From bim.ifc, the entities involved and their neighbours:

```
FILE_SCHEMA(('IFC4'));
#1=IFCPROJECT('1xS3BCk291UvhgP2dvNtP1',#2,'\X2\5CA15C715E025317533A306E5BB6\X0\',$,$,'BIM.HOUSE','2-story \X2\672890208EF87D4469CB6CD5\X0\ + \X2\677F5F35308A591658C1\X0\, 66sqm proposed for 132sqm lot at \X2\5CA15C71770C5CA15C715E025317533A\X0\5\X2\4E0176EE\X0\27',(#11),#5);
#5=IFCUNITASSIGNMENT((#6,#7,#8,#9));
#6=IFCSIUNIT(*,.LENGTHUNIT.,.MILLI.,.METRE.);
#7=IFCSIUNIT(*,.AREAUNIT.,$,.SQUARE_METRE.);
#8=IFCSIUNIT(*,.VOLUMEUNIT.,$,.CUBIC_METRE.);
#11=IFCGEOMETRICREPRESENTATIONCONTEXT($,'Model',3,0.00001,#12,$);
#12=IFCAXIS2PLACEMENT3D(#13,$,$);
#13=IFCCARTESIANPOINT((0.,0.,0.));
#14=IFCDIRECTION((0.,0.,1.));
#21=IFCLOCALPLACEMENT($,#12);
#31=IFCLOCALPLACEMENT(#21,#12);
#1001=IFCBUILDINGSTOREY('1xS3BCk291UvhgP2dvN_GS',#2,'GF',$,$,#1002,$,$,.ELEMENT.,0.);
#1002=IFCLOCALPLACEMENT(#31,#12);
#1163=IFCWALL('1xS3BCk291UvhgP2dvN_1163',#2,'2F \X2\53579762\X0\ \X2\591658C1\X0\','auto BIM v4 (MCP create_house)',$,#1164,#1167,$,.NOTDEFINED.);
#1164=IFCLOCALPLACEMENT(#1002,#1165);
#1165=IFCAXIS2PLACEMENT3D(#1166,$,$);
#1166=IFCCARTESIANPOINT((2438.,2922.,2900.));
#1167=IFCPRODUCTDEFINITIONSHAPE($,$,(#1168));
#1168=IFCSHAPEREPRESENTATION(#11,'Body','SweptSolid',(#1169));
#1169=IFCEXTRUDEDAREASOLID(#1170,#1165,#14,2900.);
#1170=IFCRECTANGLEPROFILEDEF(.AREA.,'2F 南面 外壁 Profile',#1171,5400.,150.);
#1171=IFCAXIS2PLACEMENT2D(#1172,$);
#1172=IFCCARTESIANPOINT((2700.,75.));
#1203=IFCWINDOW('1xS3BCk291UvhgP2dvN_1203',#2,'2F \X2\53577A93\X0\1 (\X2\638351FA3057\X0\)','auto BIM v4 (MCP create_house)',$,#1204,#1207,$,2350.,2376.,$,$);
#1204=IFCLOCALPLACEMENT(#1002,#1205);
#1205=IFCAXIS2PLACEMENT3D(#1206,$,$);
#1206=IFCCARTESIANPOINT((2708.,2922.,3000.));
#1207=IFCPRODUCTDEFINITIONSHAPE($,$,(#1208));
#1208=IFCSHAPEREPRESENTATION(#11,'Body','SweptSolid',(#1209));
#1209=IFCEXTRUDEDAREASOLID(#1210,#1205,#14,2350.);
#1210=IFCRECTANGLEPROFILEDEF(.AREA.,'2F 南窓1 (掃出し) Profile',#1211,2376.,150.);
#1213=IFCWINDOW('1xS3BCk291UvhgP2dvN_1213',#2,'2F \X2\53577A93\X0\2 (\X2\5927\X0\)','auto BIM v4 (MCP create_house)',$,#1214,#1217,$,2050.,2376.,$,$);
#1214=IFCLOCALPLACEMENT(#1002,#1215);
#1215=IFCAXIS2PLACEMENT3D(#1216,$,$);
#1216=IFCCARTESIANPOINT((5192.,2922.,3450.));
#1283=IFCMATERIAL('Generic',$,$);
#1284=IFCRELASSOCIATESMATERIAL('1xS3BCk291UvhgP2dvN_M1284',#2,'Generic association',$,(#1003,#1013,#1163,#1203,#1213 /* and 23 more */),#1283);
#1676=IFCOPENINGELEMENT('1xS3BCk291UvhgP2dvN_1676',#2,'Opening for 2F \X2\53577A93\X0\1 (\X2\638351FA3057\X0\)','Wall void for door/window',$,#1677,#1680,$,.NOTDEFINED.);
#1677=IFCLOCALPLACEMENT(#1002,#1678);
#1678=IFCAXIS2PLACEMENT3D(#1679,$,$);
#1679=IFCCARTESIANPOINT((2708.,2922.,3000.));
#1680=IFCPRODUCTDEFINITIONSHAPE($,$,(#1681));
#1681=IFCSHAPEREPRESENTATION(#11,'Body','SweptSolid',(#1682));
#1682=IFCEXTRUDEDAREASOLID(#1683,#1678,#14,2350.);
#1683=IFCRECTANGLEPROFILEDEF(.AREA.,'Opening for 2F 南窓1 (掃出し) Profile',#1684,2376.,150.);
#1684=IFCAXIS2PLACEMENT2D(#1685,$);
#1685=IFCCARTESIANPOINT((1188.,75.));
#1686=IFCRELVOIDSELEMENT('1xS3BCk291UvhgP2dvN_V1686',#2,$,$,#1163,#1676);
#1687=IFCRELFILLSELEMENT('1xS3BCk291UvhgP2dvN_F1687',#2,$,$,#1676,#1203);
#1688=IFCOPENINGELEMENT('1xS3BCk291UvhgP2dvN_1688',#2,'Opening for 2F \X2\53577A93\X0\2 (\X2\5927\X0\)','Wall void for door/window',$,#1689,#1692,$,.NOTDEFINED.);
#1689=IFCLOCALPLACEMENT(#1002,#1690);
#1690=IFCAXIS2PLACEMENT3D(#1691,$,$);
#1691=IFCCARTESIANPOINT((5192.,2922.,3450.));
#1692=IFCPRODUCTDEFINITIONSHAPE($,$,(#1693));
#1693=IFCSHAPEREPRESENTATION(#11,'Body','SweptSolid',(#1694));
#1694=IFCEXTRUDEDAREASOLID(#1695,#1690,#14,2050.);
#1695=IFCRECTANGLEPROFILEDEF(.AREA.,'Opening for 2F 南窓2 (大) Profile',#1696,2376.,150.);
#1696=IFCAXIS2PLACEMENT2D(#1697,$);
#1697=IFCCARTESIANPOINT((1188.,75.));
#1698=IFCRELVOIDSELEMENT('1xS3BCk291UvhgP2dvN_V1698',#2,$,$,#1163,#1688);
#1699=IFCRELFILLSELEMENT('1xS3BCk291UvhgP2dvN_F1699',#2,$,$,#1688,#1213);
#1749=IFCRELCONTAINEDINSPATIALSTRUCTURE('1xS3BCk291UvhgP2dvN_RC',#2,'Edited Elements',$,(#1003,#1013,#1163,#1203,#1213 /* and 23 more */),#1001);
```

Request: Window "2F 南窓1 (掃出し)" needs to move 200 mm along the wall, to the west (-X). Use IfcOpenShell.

```python
import ifcopenshell
import ifcopenshell.api.geometry
import ifcopenshell.util.placement
import ifcopenshell.util.unit

model = ifcopenshell.open("bim.ifc")
unit_scale = ifcopenshell.util.unit.calculate_unit_scale(model)

window = model.by_guid("1xS3BCk291UvhgP2dvN_1203")
opening = window.FillsVoids[0].RelatingOpeningElement
wall = opening.VoidsElements[0].RelatingBuildingElement

wall_matrix = ifcopenshell.util.placement.get_local_placement(wall.ObjectPlacement)
shift = wall_matrix[:3, 0] * -0.2 / unit_scale
before = ifcopenshell.util.placement.get_local_placement(window.ObjectPlacement)[:3, 3].copy()

# The window is not placed relative to its opening, so move both.
for product in (opening, window):
    matrix = ifcopenshell.util.placement.get_local_placement(product.ObjectPlacement)
    matrix[:3, 3] += shift
    ifcopenshell.api.geometry.edit_object_placement(model, product=product, matrix=matrix, is_si=False)

after = ifcopenshell.util.placement.get_local_placement(window.ObjectPlacement)[:3, 3]
print("window moved by", (after - before).round(3) + 0.0)

model.write("bim_edited.ifc")
```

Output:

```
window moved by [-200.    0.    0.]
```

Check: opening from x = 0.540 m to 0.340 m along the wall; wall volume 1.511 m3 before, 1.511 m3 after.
